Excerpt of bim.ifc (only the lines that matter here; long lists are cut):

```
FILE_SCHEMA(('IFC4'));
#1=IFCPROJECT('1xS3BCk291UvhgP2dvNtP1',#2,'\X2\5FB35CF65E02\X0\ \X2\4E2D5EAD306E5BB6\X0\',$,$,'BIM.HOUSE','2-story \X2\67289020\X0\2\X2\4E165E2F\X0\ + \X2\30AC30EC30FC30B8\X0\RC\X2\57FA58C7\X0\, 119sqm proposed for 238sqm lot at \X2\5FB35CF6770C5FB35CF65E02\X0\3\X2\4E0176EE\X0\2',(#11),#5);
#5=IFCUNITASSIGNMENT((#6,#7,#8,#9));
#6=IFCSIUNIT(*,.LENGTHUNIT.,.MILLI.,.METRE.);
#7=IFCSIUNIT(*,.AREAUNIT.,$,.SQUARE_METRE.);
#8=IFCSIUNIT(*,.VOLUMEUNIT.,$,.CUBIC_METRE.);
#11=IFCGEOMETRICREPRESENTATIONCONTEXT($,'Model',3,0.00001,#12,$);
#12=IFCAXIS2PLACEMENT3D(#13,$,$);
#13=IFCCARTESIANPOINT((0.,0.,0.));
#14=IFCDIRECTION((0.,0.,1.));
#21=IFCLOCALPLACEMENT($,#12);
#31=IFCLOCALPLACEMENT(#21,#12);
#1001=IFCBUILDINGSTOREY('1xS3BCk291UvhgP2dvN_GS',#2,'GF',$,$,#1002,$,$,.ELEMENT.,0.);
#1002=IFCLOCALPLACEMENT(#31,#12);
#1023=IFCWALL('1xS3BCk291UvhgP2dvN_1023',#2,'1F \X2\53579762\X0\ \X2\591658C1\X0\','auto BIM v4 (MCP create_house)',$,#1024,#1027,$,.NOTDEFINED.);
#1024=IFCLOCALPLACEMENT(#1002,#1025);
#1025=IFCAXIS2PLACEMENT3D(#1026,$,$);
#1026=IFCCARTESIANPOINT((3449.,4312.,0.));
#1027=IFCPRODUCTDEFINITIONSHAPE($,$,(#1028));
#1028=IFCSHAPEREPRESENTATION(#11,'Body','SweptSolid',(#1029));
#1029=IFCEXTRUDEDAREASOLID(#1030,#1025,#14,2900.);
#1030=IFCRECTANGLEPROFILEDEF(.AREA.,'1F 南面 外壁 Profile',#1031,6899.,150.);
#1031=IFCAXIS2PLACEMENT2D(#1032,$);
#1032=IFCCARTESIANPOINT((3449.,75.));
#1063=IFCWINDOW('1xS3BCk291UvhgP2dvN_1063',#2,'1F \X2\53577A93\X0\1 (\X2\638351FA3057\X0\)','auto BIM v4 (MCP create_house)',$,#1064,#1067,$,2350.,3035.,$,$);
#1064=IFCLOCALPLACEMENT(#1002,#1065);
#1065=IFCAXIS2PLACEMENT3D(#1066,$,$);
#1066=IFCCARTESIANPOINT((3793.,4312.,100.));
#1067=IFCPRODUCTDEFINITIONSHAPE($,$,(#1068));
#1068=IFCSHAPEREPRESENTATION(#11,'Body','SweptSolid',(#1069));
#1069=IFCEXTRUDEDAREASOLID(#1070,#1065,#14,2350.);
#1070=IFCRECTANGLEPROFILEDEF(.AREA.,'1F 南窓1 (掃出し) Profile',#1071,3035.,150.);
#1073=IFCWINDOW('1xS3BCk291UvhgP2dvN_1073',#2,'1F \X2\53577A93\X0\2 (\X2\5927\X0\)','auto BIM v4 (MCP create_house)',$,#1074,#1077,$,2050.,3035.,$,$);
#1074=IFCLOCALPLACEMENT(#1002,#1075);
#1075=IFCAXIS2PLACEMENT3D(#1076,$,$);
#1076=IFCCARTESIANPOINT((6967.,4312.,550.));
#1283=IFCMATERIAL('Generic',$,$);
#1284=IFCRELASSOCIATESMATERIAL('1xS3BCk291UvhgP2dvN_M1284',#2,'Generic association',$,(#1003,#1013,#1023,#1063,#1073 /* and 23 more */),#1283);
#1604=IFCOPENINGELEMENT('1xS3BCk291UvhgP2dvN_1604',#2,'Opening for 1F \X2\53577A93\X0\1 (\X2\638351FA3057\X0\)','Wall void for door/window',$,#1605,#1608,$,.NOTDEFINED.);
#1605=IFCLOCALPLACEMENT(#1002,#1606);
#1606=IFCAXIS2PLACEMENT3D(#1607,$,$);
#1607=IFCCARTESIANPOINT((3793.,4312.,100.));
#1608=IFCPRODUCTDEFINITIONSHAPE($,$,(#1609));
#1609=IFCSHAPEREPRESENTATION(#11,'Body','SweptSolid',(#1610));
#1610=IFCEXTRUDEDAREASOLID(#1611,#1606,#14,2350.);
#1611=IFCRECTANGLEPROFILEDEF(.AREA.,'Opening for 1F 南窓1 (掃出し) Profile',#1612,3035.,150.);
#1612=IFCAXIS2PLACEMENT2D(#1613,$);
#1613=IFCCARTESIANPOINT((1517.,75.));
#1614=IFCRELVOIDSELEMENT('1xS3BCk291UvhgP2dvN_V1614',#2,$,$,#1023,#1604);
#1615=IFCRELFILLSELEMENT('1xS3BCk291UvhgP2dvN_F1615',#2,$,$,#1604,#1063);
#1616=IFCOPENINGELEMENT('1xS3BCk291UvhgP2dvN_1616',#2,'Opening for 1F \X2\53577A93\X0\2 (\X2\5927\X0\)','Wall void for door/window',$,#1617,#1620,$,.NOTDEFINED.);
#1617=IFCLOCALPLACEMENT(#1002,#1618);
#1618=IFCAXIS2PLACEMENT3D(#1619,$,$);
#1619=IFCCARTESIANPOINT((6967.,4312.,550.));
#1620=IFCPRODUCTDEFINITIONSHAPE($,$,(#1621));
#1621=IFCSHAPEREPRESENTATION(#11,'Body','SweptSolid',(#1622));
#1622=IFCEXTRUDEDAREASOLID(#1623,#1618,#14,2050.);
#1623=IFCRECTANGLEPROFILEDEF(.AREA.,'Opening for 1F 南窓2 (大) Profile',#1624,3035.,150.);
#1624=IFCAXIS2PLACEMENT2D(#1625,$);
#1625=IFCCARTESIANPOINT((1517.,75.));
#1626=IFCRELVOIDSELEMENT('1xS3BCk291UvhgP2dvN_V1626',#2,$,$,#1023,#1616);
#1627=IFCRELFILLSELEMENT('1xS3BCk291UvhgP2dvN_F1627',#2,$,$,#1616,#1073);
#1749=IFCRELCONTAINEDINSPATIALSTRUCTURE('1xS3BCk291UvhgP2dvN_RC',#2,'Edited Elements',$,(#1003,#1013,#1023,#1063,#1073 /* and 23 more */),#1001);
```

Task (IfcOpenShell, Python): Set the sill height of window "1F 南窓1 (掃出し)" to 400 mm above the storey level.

```python
import numpy as np
import ifcopenshell
import ifcopenshell.api.geometry
import ifcopenshell.geom
import ifcopenshell.util.element
import ifcopenshell.util.placement
import ifcopenshell.util.shape
import ifcopenshell.util.unit

model = ifcopenshell.open("bim.ifc")
unit_scale = ifcopenshell.util.unit.calculate_unit_scale(model)

window = model.by_guid("1xS3BCk291UvhgP2dvN_1063")
opening = window.FillsVoids[0].RelatingOpeningElement
storey = ifcopenshell.util.element.get_container(window, ifc_class="IfcBuildingStorey")
level = ifcopenshell.util.placement.get_local_placement(storey.ObjectPlacement)[2, 3]

# The opening's origin need not be at the sill, so measure its lowest point.
shape = ifcopenshell.geom.create_shape(ifcopenshell.geom.settings(), opening)
bottom = ifcopenshell.util.shape.get_shape_bottom_elevation(shape, shape.geometry) / unit_scale
dz = level + 400.0 - bottom

shift = np.array([0.0, 0.0, dz])
# The window is not placed relative to its opening, so move both.
for product in (opening, window):
    matrix = ifcopenshell.util.placement.get_local_placement(product.ObjectPlacement)
    matrix[:3, 3] += shift
    ifcopenshell.api.geometry.edit_object_placement(model, product=product, matrix=matrix, is_si=False)

print(f"moved by {dz * unit_scale:+.3f} m")

model.write("bim_rev.ifc")
```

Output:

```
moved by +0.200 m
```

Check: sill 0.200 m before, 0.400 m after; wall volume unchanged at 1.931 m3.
